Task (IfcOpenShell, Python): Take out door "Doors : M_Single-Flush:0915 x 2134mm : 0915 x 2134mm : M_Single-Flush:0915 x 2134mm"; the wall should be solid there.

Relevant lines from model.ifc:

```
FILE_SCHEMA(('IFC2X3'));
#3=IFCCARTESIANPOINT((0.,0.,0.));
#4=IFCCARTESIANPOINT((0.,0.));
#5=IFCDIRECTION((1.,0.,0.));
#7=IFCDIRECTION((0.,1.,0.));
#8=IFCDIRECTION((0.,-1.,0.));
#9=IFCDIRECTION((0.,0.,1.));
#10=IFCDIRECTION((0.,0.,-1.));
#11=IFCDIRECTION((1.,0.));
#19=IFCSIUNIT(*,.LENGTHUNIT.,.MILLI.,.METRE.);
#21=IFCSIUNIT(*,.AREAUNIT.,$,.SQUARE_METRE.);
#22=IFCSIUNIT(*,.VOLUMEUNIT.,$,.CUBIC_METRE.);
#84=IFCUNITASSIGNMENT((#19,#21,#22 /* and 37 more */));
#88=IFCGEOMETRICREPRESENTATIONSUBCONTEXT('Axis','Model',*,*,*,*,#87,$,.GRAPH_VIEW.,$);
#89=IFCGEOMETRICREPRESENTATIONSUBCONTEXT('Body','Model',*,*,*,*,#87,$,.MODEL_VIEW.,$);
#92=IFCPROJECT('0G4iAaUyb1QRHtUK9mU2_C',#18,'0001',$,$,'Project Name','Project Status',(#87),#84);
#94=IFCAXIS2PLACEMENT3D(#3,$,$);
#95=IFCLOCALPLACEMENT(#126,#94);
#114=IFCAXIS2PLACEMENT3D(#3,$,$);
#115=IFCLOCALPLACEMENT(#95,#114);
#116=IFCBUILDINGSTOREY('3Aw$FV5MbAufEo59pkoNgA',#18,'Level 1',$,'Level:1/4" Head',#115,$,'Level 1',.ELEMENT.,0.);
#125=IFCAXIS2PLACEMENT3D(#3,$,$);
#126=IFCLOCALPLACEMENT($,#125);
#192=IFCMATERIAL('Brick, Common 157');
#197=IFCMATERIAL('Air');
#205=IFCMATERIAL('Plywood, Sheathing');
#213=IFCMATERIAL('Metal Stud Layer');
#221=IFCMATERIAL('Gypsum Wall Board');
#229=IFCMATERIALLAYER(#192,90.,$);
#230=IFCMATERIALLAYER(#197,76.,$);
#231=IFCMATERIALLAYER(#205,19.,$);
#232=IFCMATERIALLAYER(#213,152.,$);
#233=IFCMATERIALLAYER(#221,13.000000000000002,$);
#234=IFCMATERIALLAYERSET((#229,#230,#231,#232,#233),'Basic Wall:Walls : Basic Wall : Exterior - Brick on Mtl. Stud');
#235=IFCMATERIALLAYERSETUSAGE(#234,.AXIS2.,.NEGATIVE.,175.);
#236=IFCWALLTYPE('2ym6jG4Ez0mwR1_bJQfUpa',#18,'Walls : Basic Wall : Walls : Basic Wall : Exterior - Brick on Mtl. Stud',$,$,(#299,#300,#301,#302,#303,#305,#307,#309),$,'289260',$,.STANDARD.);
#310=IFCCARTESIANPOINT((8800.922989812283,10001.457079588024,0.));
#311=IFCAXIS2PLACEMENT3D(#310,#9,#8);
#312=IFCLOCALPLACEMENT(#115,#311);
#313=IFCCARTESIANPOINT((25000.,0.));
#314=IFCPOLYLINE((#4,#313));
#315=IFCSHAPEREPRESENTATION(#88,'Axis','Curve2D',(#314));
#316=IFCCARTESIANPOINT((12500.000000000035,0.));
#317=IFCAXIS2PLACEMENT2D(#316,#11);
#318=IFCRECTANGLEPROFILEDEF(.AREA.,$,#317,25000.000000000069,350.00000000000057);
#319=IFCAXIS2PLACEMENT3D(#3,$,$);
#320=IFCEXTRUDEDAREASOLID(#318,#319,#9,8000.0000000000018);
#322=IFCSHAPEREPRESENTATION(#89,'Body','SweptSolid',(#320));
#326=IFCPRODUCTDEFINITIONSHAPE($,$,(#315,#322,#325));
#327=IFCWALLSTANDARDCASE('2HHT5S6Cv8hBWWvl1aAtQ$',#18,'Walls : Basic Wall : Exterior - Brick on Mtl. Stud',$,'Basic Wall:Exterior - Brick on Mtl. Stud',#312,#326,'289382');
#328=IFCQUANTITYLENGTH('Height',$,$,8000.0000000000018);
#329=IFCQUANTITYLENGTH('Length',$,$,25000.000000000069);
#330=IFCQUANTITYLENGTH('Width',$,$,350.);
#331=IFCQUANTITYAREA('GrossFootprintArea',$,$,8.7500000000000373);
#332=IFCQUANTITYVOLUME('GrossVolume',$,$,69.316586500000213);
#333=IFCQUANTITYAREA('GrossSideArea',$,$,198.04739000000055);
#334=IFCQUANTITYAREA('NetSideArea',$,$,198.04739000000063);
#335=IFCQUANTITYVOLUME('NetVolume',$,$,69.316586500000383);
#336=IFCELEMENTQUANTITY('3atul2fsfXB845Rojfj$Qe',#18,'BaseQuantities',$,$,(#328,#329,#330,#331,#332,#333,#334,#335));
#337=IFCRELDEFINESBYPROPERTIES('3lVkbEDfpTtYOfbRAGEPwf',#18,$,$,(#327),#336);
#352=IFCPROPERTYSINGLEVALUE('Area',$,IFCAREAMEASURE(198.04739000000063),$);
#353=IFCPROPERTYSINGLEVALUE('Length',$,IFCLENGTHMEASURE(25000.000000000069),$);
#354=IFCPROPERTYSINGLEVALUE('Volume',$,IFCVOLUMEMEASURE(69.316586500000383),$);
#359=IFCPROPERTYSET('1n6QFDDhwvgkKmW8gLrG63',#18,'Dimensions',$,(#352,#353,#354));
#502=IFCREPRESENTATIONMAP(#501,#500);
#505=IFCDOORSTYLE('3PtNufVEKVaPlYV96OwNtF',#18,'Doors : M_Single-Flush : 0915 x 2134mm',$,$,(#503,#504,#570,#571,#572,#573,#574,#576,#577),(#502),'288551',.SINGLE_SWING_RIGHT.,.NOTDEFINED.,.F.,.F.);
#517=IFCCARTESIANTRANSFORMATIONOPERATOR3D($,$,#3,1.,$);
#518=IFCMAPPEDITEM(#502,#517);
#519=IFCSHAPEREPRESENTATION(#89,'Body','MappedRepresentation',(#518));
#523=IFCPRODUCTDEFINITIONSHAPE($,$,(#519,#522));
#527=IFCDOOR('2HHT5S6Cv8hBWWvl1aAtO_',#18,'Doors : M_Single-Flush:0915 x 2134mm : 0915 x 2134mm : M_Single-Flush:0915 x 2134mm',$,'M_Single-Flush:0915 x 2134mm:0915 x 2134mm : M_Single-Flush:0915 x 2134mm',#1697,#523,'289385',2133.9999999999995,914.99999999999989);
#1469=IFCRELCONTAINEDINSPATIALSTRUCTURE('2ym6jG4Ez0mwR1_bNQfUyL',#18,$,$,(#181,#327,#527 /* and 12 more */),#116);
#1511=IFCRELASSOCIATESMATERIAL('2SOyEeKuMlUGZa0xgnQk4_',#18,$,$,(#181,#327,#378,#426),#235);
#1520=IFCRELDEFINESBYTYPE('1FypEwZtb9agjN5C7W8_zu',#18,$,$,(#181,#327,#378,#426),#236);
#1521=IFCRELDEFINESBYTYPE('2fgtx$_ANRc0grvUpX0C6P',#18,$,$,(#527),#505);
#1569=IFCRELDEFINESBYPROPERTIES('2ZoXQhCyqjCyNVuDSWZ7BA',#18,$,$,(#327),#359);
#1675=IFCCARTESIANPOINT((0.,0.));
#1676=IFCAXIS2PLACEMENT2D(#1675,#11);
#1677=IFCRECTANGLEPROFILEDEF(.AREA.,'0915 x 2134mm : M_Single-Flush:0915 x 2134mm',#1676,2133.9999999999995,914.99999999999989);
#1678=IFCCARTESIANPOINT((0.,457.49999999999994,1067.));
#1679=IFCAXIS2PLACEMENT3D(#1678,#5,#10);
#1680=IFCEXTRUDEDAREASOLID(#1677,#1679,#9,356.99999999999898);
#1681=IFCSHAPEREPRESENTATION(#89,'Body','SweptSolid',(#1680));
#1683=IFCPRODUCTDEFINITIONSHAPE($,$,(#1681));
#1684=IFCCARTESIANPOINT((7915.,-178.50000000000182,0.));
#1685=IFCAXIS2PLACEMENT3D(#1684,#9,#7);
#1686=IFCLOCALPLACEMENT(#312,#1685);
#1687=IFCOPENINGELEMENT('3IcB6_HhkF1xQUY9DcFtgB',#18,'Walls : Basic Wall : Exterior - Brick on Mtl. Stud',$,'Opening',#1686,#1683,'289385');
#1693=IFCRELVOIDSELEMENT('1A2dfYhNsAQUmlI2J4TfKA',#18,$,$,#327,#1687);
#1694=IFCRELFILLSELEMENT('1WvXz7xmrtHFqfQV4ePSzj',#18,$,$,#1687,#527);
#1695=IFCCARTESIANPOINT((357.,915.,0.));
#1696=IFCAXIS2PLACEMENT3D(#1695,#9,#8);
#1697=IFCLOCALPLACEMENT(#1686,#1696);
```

```python
import ifcopenshell
import ifcopenshell.api.feature
import ifcopenshell.api.pset
import ifcopenshell.api.root
import ifcopenshell.geom
import ifcopenshell.util.element
import ifcopenshell.util.shape
import ifcopenshell.util.unit

model = ifcopenshell.open("model.ifc")
area_scale = ifcopenshell.util.unit.calculate_unit_scale(model, "AREAUNIT")
volume_scale = ifcopenshell.util.unit.calculate_unit_scale(model, "VOLUMEUNIT")
settings = ifcopenshell.geom.settings()


def volume(element):
    """Net volume in cubic metres, openings subtracted."""
    shape = ifcopenshell.geom.create_shape(settings, element)
    return ifcopenshell.util.shape.get_volume(shape.geometry)


door = model.by_id(527)
opening = door.FillsVoids[0].RelatingOpeningElement
wall = opening.VoidsElements[0].RelatingBuildingElement
before = volume(wall)

ifcopenshell.api.root.remove_product(model, product=door)
ifcopenshell.api.feature.remove_feature(model, feature=opening)

after = volume(wall)
thickness = 0.35  # wall thickness in metres

# Update the wall's stored quantities.
qto = model.by_id(ifcopenshell.util.element.get_pset(wall, "BaseQuantities", should_inherit=False)["id"])
ifcopenshell.api.pset.edit_qto(model, qto=qto, properties={
    "NetSideArea": after / thickness / area_scale,
    "NetVolume": after / volume_scale,
})
pset = model.by_id(ifcopenshell.util.element.get_pset(wall, "Dimensions", should_inherit=False)["id"])
ifcopenshell.api.pset.edit_pset(model, pset=pset, properties={
    "Area": model.create_entity("IfcAreaMeasure", after / thickness / area_scale),
    "Volume": model.create_entity("IfcVolumeMeasure", after / volume_scale),
})

print(f"wall volume {before:.3f} -> {after:.3f} m3")

model.write("model-out.ifc")
```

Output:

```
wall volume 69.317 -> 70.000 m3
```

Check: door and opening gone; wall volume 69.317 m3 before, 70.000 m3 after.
